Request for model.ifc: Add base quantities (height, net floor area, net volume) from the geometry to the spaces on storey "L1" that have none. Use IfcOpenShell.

First a look at what the model holds.

```python
import ifcopenshell
import ifcopenshell.util.element
import ifcopenshell.util.unit

model = ifcopenshell.open("model.ifc")
print(model.schema)
for unit_type in ("LENGTHUNIT", "AREAUNIT", "VOLUMEUNIT"):
    print(unit_type, ifcopenshell.util.unit.calculate_unit_scale(model, unit_type))
storey = next(s for s in model.by_type("IfcBuildingStorey") if s.Name == "L1")
spaces = [e for e in ifcopenshell.util.element.get_decomposition(storey) if e.is_a("IfcSpace")]
for e in sorted(spaces, key=lambda e: e.id()):
    print(e.id(), e.is_a(), e.Name, list(ifcopenshell.util.element.get_psets(e, qtos_only=True)), sep=" | ")
```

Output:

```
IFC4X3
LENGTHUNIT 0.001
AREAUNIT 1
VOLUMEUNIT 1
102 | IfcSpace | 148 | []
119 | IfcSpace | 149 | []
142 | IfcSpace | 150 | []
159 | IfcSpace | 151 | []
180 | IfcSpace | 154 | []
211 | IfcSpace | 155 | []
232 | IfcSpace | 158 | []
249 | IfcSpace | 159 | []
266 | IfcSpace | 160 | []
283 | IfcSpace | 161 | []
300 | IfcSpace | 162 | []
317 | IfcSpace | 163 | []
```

```python
import ifcopenshell
import ifcopenshell.api.pset
import ifcopenshell.geom
import ifcopenshell.util.element
import ifcopenshell.util.shape
import ifcopenshell.util.unit

model = ifcopenshell.open("model.ifc")
unit_scale = ifcopenshell.util.unit.calculate_unit_scale(model)
area_scale = ifcopenshell.util.unit.calculate_unit_scale(model, "AREAUNIT")
volume_scale = ifcopenshell.util.unit.calculate_unit_scale(model, "VOLUMEUNIT")
settings = ifcopenshell.geom.settings()

storey = next(s for s in model.by_type("IfcBuildingStorey") if s.Name == "L1")
spaces = [e for e in ifcopenshell.util.element.get_decomposition(storey) if e.is_a("IfcSpace")]

for e in sorted(spaces, key=lambda e: e.id()):
    if ifcopenshell.util.element.get_psets(e, qtos_only=True, should_inherit=False):
        continue
    # Geometry comes back in metres, in the element's own axes.
    shape = ifcopenshell.geom.create_shape(settings, e)
    values = {
        "Height": ifcopenshell.util.shape.get_z(shape.geometry) / unit_scale,
        "NetFloorArea": ifcopenshell.util.shape.get_footprint_area(shape.geometry) / area_scale,
        "NetVolume": ifcopenshell.util.shape.get_volume(shape.geometry) / volume_scale,
    }
    qto = ifcopenshell.api.pset.add_qto(model, product=e, name="Qto_SpaceBaseQuantities")
    ifcopenshell.api.pset.edit_qto(model, qto=qto, properties=values)
    print(e.id(), {k: round(v, 3) for k, v in values.items()})

model.write("model_edited.ifc")
```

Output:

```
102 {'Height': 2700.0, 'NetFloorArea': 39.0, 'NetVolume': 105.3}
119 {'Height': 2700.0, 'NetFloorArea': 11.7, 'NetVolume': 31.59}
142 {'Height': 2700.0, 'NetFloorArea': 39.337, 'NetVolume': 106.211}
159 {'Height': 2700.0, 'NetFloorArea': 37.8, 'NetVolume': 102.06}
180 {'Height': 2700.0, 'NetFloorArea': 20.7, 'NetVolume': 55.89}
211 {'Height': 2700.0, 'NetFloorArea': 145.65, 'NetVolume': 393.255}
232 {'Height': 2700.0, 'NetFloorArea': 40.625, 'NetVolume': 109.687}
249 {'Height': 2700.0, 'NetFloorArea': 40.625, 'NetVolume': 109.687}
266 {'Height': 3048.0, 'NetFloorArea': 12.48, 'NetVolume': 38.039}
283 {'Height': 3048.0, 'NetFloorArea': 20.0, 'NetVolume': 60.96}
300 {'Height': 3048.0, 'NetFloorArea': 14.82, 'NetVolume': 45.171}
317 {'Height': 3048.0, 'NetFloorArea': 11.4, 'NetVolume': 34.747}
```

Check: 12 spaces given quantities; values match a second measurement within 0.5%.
